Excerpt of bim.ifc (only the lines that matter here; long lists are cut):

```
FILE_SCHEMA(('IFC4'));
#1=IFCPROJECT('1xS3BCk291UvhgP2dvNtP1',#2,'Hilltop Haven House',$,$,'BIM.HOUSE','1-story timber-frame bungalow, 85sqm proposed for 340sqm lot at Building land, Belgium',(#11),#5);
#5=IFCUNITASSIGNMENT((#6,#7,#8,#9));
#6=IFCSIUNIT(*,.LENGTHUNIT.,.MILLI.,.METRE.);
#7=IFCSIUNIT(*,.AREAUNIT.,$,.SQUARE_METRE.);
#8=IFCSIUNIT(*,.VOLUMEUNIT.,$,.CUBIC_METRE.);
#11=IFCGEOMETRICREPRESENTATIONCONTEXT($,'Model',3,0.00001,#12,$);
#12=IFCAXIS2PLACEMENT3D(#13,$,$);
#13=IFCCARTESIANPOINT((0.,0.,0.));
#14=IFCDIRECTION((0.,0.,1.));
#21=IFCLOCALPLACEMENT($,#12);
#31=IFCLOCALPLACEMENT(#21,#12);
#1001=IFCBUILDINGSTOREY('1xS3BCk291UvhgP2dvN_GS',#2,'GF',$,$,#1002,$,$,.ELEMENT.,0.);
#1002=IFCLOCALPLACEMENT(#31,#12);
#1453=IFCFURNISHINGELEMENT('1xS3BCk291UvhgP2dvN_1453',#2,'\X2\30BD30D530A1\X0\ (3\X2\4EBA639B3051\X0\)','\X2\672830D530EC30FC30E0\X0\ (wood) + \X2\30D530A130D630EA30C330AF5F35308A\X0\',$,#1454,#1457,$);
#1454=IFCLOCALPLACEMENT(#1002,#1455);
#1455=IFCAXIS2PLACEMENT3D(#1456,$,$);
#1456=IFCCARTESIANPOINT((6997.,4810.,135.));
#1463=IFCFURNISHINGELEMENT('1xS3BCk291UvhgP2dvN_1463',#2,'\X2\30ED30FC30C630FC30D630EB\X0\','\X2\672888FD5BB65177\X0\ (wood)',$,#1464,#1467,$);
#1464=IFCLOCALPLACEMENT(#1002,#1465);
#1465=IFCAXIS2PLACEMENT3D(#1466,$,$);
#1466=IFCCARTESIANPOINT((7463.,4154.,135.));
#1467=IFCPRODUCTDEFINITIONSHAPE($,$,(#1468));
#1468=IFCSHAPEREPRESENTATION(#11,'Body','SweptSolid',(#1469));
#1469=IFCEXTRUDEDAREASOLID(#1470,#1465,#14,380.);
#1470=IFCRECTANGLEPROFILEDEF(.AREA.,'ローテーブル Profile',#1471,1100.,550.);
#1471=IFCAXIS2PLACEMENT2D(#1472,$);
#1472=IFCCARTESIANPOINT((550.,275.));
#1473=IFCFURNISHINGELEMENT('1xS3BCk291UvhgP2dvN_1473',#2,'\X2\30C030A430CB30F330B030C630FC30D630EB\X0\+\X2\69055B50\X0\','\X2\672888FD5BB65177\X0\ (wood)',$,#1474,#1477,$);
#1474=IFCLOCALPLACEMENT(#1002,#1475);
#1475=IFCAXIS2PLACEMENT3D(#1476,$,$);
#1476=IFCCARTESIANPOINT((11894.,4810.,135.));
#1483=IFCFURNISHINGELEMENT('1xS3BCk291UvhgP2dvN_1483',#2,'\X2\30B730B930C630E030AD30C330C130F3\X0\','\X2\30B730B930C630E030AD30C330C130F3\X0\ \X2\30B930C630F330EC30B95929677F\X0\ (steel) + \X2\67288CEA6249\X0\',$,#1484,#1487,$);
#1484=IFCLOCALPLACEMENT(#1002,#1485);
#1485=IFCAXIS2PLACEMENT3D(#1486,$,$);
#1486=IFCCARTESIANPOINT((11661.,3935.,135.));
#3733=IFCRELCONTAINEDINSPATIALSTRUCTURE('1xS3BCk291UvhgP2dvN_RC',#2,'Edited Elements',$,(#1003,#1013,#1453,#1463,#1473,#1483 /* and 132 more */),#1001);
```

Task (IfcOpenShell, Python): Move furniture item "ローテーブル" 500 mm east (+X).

```python
import ifcopenshell
import ifcopenshell.api.geometry
import ifcopenshell.util.placement

model = ifcopenshell.open("bim.ifc")

item = model.by_guid("1xS3BCk291UvhgP2dvN_1463")
matrix = ifcopenshell.util.placement.get_local_placement(item.ObjectPlacement)
matrix[0, 3] += 500.0
ifcopenshell.api.geometry.edit_object_placement(model, product=item, matrix=matrix, is_si=False)

print(ifcopenshell.util.placement.get_local_placement(item.ObjectPlacement).round(3) + 0.0)

model.write("bim_edited.ifc")
```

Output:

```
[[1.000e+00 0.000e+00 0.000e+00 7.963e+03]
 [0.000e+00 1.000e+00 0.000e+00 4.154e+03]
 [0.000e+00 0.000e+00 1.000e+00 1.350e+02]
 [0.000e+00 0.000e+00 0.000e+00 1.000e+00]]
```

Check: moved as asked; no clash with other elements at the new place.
